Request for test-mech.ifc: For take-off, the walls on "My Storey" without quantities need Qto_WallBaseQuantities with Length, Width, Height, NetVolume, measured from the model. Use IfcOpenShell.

First a look at what the model holds.

```python
import ifcopenshell
import ifcopenshell.util.element
import ifcopenshell.util.unit

model = ifcopenshell.open("test-mech.ifc")
print(model.schema)
for unit_type in ("LENGTHUNIT", "AREAUNIT", "VOLUMEUNIT"):
    print(unit_type, ifcopenshell.util.unit.calculate_unit_scale(model, unit_type))
storey = next(s for s in model.by_type("IfcBuildingStorey") if s.Name == "My Storey")
walls = [e for e in ifcopenshell.util.element.get_decomposition(storey) if e.is_a("IfcWall")]
for e in sorted(walls, key=lambda e: e.id()):
    print(e.id(), e.is_a(), e.Name, list(ifcopenshell.util.element.get_psets(e, qtos_only=True)), sep=" | ")
```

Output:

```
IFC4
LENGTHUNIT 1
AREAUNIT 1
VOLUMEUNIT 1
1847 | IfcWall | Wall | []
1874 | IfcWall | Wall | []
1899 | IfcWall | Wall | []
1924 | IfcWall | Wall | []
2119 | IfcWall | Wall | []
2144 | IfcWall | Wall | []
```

```python
import ifcopenshell
import ifcopenshell.api.pset
import ifcopenshell.geom
import ifcopenshell.util.element
import ifcopenshell.util.shape
import ifcopenshell.util.unit

model = ifcopenshell.open("test-mech.ifc")
unit_scale = ifcopenshell.util.unit.calculate_unit_scale(model)
volume_scale = ifcopenshell.util.unit.calculate_unit_scale(model, "VOLUMEUNIT")
settings = ifcopenshell.geom.settings()

storey = next(s for s in model.by_type("IfcBuildingStorey") if s.Name == "My Storey")
walls = [e for e in ifcopenshell.util.element.get_decomposition(storey) if e.is_a("IfcWall")]

for e in sorted(walls, key=lambda e: e.id()):
    if ifcopenshell.util.element.get_psets(e, qtos_only=True, should_inherit=False):
        continue
    # Geometry comes back in metres, in the element's own axes.
    shape = ifcopenshell.geom.create_shape(settings, e)
    values = {
        "Length": ifcopenshell.util.shape.get_x(shape.geometry) / unit_scale,
        "Width": ifcopenshell.util.shape.get_y(shape.geometry) / unit_scale,
        "Height": ifcopenshell.util.shape.get_z(shape.geometry) / unit_scale,
        "NetVolume": ifcopenshell.util.shape.get_volume(shape.geometry) / volume_scale,
    }
    qto = ifcopenshell.api.pset.add_qto(model, product=e, name="Qto_WallBaseQuantities")
    ifcopenshell.api.pset.edit_qto(model, qto=qto, properties=values)
    print(e.id(), {k: round(v, 3) for k, v in values.items()})

model.write("test-mech_edited.ifc")
```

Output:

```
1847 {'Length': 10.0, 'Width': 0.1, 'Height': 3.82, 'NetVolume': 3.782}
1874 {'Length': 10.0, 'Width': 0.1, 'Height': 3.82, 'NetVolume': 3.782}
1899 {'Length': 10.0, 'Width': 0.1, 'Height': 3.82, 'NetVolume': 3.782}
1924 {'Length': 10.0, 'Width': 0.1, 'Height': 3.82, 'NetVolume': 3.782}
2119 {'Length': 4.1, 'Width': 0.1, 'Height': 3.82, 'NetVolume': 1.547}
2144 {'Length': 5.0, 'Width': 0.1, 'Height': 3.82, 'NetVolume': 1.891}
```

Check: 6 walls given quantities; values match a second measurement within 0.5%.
